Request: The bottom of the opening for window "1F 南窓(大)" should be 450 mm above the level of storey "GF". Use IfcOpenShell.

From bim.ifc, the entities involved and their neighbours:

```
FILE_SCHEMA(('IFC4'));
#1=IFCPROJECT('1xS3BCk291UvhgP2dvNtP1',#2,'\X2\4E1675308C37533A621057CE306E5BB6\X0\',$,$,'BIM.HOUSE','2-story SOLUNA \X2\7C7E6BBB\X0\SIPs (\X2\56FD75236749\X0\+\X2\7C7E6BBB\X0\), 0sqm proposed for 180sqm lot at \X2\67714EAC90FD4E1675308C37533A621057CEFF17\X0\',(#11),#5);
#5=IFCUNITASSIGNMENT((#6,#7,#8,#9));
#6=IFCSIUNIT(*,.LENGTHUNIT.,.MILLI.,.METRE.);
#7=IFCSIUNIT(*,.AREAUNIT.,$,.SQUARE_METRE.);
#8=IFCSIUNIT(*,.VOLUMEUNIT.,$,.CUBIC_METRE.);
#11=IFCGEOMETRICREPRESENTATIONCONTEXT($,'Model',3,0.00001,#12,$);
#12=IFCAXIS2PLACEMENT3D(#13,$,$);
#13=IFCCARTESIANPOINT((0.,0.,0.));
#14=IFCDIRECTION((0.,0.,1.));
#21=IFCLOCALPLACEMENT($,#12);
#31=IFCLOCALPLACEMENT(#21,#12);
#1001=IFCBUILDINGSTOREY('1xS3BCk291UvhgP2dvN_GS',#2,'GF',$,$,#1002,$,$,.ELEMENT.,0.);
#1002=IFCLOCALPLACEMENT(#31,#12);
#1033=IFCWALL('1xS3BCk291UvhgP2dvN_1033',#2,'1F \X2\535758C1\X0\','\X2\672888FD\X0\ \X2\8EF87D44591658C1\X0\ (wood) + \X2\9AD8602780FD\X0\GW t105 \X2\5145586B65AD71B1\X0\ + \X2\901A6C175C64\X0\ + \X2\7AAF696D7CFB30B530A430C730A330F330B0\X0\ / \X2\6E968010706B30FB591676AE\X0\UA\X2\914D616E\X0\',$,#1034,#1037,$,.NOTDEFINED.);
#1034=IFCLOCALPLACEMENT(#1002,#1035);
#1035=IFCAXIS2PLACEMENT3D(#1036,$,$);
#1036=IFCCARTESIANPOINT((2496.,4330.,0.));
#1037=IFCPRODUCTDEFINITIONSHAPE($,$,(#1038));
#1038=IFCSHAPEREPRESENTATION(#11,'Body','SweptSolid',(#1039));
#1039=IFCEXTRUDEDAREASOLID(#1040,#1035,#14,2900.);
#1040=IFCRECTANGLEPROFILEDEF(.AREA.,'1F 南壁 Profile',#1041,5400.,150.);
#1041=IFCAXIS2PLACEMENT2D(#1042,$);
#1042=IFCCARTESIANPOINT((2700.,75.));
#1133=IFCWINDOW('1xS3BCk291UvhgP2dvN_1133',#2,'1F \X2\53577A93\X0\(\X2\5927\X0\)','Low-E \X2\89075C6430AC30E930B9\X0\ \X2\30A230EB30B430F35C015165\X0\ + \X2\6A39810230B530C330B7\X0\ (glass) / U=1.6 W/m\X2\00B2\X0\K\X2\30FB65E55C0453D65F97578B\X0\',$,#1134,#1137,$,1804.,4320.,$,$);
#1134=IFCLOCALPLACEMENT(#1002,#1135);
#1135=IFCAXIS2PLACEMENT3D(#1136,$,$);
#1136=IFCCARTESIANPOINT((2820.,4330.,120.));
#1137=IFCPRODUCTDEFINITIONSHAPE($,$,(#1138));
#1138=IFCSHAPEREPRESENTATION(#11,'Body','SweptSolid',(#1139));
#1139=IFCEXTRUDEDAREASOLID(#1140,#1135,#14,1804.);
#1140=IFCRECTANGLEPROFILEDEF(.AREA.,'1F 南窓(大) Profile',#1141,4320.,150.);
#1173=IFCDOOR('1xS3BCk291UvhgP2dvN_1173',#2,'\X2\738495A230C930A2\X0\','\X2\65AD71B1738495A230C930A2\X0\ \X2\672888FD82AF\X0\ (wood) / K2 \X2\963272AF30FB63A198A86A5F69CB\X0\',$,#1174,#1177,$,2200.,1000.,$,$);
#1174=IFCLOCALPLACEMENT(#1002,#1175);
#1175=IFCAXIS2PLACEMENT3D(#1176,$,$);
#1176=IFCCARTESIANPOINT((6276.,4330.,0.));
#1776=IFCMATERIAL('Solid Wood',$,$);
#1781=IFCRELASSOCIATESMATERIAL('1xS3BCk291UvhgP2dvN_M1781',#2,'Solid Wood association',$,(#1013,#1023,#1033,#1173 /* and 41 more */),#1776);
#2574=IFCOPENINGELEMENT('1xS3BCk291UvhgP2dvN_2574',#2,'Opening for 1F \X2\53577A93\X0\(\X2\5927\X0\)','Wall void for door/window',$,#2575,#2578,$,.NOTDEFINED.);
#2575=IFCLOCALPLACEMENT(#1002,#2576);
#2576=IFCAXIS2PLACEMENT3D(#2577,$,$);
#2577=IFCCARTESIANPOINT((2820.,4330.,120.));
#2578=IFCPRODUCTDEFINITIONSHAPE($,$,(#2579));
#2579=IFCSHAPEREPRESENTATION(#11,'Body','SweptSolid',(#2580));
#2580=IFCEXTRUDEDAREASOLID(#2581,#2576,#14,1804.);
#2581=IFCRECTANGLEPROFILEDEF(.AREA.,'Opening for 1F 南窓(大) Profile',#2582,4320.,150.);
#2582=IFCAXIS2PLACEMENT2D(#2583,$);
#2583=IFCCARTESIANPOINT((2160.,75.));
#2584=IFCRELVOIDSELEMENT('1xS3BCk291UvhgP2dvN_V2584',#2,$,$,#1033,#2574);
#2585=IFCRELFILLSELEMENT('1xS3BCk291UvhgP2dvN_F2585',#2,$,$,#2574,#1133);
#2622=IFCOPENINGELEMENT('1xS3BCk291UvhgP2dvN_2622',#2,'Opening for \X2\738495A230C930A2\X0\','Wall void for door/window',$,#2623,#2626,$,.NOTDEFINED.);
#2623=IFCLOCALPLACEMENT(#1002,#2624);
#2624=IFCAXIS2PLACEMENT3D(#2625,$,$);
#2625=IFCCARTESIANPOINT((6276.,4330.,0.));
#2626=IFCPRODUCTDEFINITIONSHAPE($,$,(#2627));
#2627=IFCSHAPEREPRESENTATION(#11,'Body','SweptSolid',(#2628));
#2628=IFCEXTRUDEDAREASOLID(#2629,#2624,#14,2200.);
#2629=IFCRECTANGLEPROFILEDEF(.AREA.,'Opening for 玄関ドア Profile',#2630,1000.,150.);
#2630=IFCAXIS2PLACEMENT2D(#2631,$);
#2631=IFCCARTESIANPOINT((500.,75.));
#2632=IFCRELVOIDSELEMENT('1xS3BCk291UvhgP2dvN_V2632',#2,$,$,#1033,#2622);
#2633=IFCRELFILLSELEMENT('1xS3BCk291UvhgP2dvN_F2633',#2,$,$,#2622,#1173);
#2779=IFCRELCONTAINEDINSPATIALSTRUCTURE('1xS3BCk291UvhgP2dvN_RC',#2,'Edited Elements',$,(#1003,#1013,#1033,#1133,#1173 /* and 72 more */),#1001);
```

```python
import numpy as np
import ifcopenshell
import ifcopenshell.api.geometry
import ifcopenshell.geom
import ifcopenshell.util.element
import ifcopenshell.util.placement
import ifcopenshell.util.shape
import ifcopenshell.util.unit

model = ifcopenshell.open("bim.ifc")
unit_scale = ifcopenshell.util.unit.calculate_unit_scale(model)

window = model.by_guid("1xS3BCk291UvhgP2dvN_1133")
opening = window.FillsVoids[0].RelatingOpeningElement
storey = ifcopenshell.util.element.get_container(window, ifc_class="IfcBuildingStorey")
level = ifcopenshell.util.placement.get_local_placement(storey.ObjectPlacement)[2, 3]

# The opening's origin need not be at the sill, so measure its lowest point.
shape = ifcopenshell.geom.create_shape(ifcopenshell.geom.settings(), opening)
bottom = ifcopenshell.util.shape.get_shape_bottom_elevation(shape, shape.geometry) / unit_scale
dz = level + 0.45 / unit_scale - bottom

shift = np.array([0.0, 0.0, dz])
# The window is not placed relative to its opening, so move both.
for product in (opening, window):
    matrix = ifcopenshell.util.placement.get_local_placement(product.ObjectPlacement)
    matrix[:3, 3] += shift
    ifcopenshell.api.geometry.edit_object_placement(model, product=product, matrix=matrix, is_si=False)

print(f"moved by {dz * unit_scale:+.3f} m")

model.write("bim_edited.ifc")
```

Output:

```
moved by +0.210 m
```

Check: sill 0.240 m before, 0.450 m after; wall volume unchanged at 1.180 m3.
